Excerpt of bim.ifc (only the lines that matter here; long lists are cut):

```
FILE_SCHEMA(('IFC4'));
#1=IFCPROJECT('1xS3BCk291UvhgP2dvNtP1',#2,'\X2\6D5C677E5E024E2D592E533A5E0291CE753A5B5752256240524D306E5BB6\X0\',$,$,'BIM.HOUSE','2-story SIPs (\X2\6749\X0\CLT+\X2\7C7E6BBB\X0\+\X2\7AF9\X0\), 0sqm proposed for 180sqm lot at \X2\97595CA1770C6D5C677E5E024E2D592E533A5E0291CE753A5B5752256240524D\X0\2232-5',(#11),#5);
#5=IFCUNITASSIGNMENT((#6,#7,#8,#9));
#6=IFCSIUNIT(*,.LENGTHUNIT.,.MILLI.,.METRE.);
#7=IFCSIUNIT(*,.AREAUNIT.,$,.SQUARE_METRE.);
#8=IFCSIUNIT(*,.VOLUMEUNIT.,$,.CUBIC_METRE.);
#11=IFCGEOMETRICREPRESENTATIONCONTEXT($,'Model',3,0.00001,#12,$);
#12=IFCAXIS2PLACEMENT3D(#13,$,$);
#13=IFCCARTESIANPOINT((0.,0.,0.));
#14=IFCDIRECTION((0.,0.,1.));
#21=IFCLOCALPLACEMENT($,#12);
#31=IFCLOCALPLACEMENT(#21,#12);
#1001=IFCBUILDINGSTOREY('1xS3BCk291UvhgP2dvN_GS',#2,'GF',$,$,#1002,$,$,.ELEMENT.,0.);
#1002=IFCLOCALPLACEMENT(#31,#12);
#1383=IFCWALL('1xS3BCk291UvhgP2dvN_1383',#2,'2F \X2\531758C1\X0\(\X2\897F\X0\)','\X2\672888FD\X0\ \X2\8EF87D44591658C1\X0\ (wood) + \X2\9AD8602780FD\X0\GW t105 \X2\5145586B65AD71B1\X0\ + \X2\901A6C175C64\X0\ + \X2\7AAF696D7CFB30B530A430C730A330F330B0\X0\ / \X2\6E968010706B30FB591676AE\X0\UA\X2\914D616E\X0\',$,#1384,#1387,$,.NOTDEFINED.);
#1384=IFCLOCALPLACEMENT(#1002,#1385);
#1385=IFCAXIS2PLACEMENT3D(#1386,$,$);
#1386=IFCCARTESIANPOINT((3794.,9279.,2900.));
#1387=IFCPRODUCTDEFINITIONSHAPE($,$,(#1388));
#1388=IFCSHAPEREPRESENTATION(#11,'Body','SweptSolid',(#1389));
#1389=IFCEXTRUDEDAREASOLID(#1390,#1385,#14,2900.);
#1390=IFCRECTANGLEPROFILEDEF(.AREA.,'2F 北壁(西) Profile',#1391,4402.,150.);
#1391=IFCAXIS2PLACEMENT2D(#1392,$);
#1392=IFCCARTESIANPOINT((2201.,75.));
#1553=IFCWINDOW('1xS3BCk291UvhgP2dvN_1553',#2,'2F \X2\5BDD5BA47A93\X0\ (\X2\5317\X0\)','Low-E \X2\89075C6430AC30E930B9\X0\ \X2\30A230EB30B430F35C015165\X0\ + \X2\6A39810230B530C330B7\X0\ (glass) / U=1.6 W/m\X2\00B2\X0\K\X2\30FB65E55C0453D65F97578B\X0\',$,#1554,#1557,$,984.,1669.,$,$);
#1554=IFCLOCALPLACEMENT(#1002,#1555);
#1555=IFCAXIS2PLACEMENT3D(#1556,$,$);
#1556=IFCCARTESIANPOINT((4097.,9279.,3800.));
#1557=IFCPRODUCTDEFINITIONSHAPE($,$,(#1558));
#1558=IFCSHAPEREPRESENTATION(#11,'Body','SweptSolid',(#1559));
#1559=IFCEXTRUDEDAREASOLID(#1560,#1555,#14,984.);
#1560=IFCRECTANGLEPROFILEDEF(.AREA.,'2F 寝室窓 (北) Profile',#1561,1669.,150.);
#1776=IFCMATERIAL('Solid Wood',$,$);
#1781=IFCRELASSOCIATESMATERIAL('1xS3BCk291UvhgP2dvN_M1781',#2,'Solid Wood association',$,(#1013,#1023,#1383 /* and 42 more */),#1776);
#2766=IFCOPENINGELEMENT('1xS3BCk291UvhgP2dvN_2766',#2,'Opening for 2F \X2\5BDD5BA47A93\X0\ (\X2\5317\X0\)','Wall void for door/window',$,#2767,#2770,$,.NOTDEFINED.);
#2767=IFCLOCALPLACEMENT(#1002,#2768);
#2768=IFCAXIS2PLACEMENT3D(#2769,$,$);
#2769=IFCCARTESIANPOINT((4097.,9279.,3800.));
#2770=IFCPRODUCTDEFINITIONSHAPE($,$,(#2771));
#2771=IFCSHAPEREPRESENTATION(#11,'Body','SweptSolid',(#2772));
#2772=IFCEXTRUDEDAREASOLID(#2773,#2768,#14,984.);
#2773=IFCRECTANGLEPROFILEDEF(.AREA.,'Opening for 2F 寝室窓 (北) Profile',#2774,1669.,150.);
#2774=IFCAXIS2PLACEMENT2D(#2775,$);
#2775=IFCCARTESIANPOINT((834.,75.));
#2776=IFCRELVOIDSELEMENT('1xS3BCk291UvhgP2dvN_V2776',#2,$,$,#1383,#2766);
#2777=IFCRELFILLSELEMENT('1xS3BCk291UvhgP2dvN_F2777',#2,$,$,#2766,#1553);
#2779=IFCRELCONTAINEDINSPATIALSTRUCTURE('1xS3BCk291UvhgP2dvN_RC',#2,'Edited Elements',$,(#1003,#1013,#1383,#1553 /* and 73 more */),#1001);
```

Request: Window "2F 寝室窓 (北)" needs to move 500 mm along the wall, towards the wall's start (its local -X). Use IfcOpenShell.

```python
import ifcopenshell
import ifcopenshell.api.geometry
import ifcopenshell.util.placement
import ifcopenshell.util.unit

model = ifcopenshell.open("bim.ifc")
unit_scale = ifcopenshell.util.unit.calculate_unit_scale(model)

window = model.by_guid("1xS3BCk291UvhgP2dvN_1553")
opening = window.FillsVoids[0].RelatingOpeningElement
wall = opening.VoidsElements[0].RelatingBuildingElement

wall_matrix = ifcopenshell.util.placement.get_local_placement(wall.ObjectPlacement)
shift = wall_matrix[:3, 0] * -0.5 / unit_scale
before = ifcopenshell.util.placement.get_local_placement(window.ObjectPlacement)[:3, 3].copy()

# The window is not placed relative to its opening, so move both.
for product in (opening, window):
    matrix = ifcopenshell.util.placement.get_local_placement(product.ObjectPlacement)
    matrix[:3, 3] += shift
    ifcopenshell.api.geometry.edit_object_placement(model, product=product, matrix=matrix, is_si=False)

after = ifcopenshell.util.placement.get_local_placement(window.ObjectPlacement)[:3, 3]
print("window moved by", (after - before).round(3) + 0.0)

model.write("bim_v2.ifc")
```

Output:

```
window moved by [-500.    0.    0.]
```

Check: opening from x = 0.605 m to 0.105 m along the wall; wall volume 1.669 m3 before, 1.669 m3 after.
